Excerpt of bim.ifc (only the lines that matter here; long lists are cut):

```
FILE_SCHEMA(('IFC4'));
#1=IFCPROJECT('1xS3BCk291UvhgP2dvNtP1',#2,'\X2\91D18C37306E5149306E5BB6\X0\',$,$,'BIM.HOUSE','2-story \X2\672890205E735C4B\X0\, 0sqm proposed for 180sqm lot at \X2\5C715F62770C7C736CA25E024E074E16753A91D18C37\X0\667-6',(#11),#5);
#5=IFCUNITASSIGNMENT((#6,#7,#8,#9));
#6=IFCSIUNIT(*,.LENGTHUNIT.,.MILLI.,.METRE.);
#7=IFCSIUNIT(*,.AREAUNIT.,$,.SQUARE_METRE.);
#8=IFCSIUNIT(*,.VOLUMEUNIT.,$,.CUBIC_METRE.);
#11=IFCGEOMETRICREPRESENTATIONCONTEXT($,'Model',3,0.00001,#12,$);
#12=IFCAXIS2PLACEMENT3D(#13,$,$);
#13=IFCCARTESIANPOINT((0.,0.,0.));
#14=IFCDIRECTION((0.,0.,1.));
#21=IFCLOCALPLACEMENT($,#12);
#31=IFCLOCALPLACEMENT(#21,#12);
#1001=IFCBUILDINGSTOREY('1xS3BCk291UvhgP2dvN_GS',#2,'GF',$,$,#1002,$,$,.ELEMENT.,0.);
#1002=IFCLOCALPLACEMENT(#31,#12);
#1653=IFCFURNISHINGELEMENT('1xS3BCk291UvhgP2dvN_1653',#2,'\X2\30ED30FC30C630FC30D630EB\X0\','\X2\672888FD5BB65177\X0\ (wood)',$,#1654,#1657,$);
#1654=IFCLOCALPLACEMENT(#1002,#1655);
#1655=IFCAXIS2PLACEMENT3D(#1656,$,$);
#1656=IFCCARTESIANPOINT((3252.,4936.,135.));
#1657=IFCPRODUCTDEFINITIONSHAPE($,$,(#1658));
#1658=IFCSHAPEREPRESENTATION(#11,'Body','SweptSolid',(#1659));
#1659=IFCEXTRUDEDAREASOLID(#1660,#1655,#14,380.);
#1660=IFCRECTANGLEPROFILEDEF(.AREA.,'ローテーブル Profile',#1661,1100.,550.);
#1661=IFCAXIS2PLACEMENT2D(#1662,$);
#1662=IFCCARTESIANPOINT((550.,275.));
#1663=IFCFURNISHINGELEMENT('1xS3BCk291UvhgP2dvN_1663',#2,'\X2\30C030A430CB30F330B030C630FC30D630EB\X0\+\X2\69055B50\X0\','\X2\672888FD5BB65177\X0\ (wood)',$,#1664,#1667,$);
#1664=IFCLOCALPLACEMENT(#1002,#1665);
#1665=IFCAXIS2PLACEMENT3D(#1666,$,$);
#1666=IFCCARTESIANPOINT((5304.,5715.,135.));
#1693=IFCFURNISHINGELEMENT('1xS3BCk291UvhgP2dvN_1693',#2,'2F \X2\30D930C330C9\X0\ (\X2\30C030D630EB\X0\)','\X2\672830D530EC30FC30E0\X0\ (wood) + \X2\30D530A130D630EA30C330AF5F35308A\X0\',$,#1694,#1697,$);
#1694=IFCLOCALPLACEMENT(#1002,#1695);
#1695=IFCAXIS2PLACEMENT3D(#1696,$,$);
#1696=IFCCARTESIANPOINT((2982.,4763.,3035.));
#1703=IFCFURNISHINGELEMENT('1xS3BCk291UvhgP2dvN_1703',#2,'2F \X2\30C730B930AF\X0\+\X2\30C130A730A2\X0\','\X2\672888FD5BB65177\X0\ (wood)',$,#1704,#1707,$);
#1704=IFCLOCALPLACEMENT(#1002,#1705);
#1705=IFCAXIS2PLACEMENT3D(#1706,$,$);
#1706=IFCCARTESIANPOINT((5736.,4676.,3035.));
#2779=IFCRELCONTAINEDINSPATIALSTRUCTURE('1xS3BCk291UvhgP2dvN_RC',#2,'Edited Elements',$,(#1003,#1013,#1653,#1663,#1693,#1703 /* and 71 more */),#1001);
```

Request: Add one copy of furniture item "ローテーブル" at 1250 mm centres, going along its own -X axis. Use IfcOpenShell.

```python
import ifcopenshell
import ifcopenshell.api.geometry
import ifcopenshell.api.root
import ifcopenshell.util.element
import ifcopenshell.util.placement

model = ifcopenshell.open("bim.ifc")


def reuse_history(source, copy):
    """copy_class also copies each property set's owner history, people and application; keep the originals."""
    for rel in copy.IsDefinedBy:
        if rel.is_a("IfcRelDefinesByProperties") and (history := rel.RelatingPropertyDefinition.OwnerHistory):
            rel.RelatingPropertyDefinition.OwnerHistory = source.OwnerHistory
            ifcopenshell.util.element.remove_deep2(model, history)


source = model.by_guid("1xS3BCk291UvhgP2dvN_1653")
base = ifcopenshell.util.placement.get_local_placement(source.ObjectPlacement)
step = -base[:3, 0] * 1250.0

for i in range(1, 2):
    copy = ifcopenshell.api.root.copy_class(model, product=source)
    copy.Representation = ifcopenshell.util.element.copy_deep(
        model, source.Representation, exclude=["IfcGeometricRepresentationContext", "IfcRepresentationMap"]
    )
    reuse_history(source, copy)
    matrix = base.copy()
    matrix[:3, 3] += i * step
    print("added at", matrix[:3, 3].round(3) + 0.0)
    ifcopenshell.api.geometry.edit_object_placement(model, product=copy, matrix=matrix, is_si=False)

model.write("bim_rev.ifc")
```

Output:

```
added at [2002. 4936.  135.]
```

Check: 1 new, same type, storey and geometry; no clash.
